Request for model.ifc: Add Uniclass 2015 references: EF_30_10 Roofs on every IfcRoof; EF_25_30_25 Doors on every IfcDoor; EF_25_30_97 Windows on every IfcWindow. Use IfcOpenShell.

First a look at what the model holds.

```python
import ifcopenshell

model = ifcopenshell.open("model.ifc")
print(model.schema)
print("classifications:", [c.Name for c in model.by_type("IfcClassification")])
for ifc_class in ("IfcDoor", "IfcRoof", "IfcStair", "IfcWall", "IfcWindow"):
    print(ifc_class, len(model.by_type(ifc_class)))
```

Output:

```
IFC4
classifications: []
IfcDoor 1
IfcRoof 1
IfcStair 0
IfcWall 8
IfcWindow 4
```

```python
import ifcopenshell
import ifcopenshell.api.classification

model = ifcopenshell.open("model.ifc")

system = ifcopenshell.api.classification.add_classification(model, classification="Uniclass 2015")

codes = {
    "IfcRoof": ("EF_30_10", "Roofs"),
    "IfcDoor": ("EF_25_30_25", "Doors"),
    "IfcWindow": ("EF_25_30_97", "Windows"),
}
for ifc_class, (code, name) in codes.items():
    products = model.by_type(ifc_class)
    ifcopenshell.api.classification.add_reference(
        model, products=products, classification=system, identification=code, name=name
    )
    print(code, len(products))

model.write("model-out.ifc")
```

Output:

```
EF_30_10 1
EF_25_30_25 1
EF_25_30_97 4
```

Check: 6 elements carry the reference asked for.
